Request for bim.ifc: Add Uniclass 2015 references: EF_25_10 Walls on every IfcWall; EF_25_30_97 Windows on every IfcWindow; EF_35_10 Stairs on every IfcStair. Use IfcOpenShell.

First a look at what the model holds.

```python
import ifcopenshell

model = ifcopenshell.open("bim.ifc")
print(model.schema)
print("classifications:", [c.Name for c in model.by_type("IfcClassification")])
for ifc_class in ("IfcDoor", "IfcRoof", "IfcStair", "IfcWall", "IfcWindow"):
    print(ifc_class, len(model.by_type(ifc_class)))
```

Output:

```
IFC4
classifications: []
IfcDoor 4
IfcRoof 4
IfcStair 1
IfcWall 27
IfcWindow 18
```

```python
import ifcopenshell
import ifcopenshell.api.classification

model = ifcopenshell.open("bim.ifc")

system = ifcopenshell.api.classification.add_classification(model, classification="Uniclass 2015")

codes = {
    "IfcWall": ("EF_25_10", "Walls"),
    "IfcWindow": ("EF_25_30_97", "Windows"),
    "IfcStair": ("EF_35_10", "Stairs"),
}
for ifc_class, (code, name) in codes.items():
    products = model.by_type(ifc_class)
    ifcopenshell.api.classification.add_reference(
        model, products=products, classification=system, identification=code, name=name
    )
    print(code, len(products))

model.write("bim-out.ifc")
```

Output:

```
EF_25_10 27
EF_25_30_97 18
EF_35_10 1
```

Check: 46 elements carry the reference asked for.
